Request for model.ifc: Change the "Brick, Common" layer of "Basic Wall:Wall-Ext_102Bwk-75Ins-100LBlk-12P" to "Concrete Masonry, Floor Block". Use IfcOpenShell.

First a look at what the model holds.

```python
import ifcopenshell
import ifcopenshell.util.element

model = ifcopenshell.open("model.ifc")
print(model.schema)
for layer_set in model.by_type("IfcMaterialLayerSet"):
    if layer_set.LayerSetName == "Basic Wall:Wall-Ext_102Bwk-75Ins-100LBlk-12P":
        for layer in layer_set.MaterialLayers:
            print(layer.id(), layer.Material and layer.Material.Name, layer.LayerThickness, sep=" | ")
        print(len(ifcopenshell.util.element.get_elements_by_material(model, layer_set)), "elements and types use it")
print(sorted(m.Name for m in model.by_type("IfcMaterial") if m.Name)[:60])
```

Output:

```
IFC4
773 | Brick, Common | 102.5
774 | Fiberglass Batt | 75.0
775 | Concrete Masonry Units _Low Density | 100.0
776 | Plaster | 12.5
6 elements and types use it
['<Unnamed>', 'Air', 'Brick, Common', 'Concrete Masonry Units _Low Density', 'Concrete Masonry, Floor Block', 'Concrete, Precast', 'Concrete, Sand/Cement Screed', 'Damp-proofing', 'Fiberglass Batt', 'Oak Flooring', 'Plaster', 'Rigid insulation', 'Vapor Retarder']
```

```python
import ifcopenshell
import ifcopenshell.api.material

model = ifcopenshell.open("model.ifc")

layer_set = next(s for s in model.by_type("IfcMaterialLayerSet") if s.LayerSetName == "Basic Wall:Wall-Ext_102Bwk-75Ins-100LBlk-12P")
layer = next(l for l in layer_set.MaterialLayers if l.Material and l.Material.Name == "Brick, Common")
material = next(m for m in model.by_type("IfcMaterial") if m.Name == "Concrete Masonry, Floor Block")

# Point this one layer at the other material; renaming the old one would change it everywhere.
ifcopenshell.api.material.edit_layer(model, layer=layer, attributes={"Name": material.Name}, material=material)

print([l.Material.Name if l.Material else None for l in layer_set.MaterialLayers])

model.write("model_edited.ifc")
```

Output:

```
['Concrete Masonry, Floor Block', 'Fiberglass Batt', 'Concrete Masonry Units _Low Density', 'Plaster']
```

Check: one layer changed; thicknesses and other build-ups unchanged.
